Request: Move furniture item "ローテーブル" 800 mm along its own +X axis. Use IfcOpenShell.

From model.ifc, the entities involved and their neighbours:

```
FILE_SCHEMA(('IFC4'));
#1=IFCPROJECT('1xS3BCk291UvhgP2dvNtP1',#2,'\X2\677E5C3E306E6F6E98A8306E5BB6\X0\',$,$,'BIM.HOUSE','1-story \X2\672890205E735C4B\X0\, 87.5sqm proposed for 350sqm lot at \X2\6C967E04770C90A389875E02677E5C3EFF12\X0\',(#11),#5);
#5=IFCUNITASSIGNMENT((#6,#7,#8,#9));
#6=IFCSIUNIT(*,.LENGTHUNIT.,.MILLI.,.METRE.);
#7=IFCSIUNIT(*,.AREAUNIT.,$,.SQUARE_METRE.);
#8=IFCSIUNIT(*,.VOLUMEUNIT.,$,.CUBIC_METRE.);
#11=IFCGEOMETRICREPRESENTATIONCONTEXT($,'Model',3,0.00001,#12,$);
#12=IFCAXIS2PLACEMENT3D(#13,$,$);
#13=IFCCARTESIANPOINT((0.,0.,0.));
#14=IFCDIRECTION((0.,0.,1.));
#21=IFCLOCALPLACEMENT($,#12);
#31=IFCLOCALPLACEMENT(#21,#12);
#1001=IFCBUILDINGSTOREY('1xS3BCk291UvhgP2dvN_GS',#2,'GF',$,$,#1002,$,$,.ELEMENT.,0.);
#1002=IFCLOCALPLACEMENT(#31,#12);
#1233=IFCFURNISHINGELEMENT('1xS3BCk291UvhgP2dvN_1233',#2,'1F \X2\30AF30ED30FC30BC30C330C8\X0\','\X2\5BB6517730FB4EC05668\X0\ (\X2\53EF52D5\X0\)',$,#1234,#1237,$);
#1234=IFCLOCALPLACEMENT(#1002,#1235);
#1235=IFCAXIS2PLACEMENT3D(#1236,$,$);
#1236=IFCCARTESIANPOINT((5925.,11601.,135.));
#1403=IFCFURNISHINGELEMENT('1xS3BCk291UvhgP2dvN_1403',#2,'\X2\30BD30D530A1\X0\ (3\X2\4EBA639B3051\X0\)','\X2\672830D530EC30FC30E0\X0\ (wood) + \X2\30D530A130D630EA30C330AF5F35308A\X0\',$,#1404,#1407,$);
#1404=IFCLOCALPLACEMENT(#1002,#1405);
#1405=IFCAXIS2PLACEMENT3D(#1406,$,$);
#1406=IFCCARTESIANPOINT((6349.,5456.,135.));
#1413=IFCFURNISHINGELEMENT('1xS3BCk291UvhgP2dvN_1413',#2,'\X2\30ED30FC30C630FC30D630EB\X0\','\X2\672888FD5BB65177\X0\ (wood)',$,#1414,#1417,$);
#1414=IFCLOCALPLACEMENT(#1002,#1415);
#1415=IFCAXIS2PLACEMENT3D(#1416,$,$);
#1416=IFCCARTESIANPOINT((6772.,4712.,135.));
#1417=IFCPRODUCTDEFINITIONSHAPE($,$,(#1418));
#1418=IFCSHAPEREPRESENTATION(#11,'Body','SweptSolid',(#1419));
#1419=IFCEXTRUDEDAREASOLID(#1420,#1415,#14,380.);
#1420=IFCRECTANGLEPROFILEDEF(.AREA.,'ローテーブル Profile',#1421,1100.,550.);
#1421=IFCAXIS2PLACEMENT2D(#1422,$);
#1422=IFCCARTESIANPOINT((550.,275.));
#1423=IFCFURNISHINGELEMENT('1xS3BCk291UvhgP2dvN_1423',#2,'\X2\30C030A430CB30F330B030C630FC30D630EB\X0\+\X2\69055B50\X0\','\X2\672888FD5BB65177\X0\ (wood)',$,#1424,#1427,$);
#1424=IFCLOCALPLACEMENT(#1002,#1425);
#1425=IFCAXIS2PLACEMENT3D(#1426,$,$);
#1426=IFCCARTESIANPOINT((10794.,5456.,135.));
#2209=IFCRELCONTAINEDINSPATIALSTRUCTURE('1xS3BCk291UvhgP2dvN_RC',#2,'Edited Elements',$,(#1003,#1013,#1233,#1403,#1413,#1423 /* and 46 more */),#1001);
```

```python
import ifcopenshell
import ifcopenshell.api.geometry
import ifcopenshell.util.placement
import ifcopenshell.util.unit

model = ifcopenshell.open("model.ifc")
unit_scale = ifcopenshell.util.unit.calculate_unit_scale(model)

item = model.by_guid("1xS3BCk291UvhgP2dvN_1413")
matrix = ifcopenshell.util.placement.get_local_placement(item.ObjectPlacement)
matrix[:3, 3] += matrix[:3, 0] * 0.8 / unit_scale
ifcopenshell.api.geometry.edit_object_placement(model, product=item, matrix=matrix, is_si=False)

print(ifcopenshell.util.placement.get_local_placement(item.ObjectPlacement).round(3) + 0.0)

model.write("model_rev.ifc")
```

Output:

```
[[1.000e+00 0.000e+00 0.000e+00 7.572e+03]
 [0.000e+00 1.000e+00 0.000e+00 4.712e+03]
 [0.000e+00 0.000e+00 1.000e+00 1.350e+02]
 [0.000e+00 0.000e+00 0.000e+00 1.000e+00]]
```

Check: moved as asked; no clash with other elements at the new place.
